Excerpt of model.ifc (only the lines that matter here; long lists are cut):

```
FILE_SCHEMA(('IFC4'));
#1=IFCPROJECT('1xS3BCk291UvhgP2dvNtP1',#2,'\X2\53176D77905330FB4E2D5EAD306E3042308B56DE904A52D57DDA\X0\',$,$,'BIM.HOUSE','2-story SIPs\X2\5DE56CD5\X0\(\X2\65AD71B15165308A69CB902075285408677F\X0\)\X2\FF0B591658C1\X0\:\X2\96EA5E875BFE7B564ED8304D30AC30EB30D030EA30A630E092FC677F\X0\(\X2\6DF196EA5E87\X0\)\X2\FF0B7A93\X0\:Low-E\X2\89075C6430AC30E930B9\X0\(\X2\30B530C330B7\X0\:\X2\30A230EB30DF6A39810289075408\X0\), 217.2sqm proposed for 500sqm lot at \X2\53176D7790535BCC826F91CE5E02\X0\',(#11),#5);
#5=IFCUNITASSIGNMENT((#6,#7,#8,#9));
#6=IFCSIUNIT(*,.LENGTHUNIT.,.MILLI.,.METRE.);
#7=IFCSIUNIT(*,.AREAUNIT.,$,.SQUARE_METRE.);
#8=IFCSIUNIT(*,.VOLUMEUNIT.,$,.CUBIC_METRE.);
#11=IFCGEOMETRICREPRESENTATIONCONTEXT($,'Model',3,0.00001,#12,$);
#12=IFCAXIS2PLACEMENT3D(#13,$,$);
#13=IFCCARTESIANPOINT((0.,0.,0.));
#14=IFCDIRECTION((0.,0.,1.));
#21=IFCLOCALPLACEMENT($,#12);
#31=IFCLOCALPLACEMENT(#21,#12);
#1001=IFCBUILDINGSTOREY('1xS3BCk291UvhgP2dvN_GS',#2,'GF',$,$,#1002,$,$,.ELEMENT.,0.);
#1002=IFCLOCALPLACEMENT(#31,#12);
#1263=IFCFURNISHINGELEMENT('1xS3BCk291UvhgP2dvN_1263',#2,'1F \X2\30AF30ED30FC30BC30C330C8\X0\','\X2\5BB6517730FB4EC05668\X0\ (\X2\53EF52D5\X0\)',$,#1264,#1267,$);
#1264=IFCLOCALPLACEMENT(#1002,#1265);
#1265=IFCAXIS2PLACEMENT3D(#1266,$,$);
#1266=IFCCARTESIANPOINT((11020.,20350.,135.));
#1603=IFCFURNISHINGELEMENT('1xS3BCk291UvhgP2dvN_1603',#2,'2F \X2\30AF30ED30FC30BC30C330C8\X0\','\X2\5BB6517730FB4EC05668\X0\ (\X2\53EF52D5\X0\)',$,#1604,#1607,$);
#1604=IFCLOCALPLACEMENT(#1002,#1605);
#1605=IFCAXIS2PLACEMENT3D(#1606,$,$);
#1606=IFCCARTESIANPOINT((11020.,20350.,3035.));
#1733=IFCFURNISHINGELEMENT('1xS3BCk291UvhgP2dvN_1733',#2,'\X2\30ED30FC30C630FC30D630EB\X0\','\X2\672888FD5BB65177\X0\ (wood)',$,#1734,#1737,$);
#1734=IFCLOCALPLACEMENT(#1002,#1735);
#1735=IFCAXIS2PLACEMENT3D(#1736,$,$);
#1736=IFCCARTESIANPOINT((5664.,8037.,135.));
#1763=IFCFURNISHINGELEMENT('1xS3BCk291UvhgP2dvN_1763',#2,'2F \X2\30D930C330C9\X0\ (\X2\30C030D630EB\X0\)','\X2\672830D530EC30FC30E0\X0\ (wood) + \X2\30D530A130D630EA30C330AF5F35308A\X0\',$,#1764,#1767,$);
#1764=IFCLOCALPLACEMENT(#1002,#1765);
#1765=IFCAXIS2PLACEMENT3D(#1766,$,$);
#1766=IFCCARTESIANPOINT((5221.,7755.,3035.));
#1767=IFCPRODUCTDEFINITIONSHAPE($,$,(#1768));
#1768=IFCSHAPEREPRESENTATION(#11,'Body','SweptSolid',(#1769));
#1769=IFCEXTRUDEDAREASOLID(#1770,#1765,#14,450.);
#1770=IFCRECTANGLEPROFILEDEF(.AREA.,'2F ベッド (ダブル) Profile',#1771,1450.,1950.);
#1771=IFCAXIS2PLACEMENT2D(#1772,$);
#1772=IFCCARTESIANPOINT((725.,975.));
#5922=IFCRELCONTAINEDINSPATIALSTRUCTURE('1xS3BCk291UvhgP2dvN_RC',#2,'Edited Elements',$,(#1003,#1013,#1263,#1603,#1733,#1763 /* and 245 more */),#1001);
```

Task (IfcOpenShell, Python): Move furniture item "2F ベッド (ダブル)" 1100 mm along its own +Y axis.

```python
import ifcopenshell
import ifcopenshell.api.geometry
import ifcopenshell.util.placement
import ifcopenshell.util.unit

model = ifcopenshell.open("model.ifc")
unit_scale = ifcopenshell.util.unit.calculate_unit_scale(model)

item = model.by_guid("1xS3BCk291UvhgP2dvN_1763")
matrix = ifcopenshell.util.placement.get_local_placement(item.ObjectPlacement)
matrix[:3, 3] += matrix[:3, 1] * 1.1 / unit_scale
ifcopenshell.api.geometry.edit_object_placement(model, product=item, matrix=matrix, is_si=False)

print(ifcopenshell.util.placement.get_local_placement(item.ObjectPlacement).round(3) + 0.0)

model.write("model_v2.ifc")
```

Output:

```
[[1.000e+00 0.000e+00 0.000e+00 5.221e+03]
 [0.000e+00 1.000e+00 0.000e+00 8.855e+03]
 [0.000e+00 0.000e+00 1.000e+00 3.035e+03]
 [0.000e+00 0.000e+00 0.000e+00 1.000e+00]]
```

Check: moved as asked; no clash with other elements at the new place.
